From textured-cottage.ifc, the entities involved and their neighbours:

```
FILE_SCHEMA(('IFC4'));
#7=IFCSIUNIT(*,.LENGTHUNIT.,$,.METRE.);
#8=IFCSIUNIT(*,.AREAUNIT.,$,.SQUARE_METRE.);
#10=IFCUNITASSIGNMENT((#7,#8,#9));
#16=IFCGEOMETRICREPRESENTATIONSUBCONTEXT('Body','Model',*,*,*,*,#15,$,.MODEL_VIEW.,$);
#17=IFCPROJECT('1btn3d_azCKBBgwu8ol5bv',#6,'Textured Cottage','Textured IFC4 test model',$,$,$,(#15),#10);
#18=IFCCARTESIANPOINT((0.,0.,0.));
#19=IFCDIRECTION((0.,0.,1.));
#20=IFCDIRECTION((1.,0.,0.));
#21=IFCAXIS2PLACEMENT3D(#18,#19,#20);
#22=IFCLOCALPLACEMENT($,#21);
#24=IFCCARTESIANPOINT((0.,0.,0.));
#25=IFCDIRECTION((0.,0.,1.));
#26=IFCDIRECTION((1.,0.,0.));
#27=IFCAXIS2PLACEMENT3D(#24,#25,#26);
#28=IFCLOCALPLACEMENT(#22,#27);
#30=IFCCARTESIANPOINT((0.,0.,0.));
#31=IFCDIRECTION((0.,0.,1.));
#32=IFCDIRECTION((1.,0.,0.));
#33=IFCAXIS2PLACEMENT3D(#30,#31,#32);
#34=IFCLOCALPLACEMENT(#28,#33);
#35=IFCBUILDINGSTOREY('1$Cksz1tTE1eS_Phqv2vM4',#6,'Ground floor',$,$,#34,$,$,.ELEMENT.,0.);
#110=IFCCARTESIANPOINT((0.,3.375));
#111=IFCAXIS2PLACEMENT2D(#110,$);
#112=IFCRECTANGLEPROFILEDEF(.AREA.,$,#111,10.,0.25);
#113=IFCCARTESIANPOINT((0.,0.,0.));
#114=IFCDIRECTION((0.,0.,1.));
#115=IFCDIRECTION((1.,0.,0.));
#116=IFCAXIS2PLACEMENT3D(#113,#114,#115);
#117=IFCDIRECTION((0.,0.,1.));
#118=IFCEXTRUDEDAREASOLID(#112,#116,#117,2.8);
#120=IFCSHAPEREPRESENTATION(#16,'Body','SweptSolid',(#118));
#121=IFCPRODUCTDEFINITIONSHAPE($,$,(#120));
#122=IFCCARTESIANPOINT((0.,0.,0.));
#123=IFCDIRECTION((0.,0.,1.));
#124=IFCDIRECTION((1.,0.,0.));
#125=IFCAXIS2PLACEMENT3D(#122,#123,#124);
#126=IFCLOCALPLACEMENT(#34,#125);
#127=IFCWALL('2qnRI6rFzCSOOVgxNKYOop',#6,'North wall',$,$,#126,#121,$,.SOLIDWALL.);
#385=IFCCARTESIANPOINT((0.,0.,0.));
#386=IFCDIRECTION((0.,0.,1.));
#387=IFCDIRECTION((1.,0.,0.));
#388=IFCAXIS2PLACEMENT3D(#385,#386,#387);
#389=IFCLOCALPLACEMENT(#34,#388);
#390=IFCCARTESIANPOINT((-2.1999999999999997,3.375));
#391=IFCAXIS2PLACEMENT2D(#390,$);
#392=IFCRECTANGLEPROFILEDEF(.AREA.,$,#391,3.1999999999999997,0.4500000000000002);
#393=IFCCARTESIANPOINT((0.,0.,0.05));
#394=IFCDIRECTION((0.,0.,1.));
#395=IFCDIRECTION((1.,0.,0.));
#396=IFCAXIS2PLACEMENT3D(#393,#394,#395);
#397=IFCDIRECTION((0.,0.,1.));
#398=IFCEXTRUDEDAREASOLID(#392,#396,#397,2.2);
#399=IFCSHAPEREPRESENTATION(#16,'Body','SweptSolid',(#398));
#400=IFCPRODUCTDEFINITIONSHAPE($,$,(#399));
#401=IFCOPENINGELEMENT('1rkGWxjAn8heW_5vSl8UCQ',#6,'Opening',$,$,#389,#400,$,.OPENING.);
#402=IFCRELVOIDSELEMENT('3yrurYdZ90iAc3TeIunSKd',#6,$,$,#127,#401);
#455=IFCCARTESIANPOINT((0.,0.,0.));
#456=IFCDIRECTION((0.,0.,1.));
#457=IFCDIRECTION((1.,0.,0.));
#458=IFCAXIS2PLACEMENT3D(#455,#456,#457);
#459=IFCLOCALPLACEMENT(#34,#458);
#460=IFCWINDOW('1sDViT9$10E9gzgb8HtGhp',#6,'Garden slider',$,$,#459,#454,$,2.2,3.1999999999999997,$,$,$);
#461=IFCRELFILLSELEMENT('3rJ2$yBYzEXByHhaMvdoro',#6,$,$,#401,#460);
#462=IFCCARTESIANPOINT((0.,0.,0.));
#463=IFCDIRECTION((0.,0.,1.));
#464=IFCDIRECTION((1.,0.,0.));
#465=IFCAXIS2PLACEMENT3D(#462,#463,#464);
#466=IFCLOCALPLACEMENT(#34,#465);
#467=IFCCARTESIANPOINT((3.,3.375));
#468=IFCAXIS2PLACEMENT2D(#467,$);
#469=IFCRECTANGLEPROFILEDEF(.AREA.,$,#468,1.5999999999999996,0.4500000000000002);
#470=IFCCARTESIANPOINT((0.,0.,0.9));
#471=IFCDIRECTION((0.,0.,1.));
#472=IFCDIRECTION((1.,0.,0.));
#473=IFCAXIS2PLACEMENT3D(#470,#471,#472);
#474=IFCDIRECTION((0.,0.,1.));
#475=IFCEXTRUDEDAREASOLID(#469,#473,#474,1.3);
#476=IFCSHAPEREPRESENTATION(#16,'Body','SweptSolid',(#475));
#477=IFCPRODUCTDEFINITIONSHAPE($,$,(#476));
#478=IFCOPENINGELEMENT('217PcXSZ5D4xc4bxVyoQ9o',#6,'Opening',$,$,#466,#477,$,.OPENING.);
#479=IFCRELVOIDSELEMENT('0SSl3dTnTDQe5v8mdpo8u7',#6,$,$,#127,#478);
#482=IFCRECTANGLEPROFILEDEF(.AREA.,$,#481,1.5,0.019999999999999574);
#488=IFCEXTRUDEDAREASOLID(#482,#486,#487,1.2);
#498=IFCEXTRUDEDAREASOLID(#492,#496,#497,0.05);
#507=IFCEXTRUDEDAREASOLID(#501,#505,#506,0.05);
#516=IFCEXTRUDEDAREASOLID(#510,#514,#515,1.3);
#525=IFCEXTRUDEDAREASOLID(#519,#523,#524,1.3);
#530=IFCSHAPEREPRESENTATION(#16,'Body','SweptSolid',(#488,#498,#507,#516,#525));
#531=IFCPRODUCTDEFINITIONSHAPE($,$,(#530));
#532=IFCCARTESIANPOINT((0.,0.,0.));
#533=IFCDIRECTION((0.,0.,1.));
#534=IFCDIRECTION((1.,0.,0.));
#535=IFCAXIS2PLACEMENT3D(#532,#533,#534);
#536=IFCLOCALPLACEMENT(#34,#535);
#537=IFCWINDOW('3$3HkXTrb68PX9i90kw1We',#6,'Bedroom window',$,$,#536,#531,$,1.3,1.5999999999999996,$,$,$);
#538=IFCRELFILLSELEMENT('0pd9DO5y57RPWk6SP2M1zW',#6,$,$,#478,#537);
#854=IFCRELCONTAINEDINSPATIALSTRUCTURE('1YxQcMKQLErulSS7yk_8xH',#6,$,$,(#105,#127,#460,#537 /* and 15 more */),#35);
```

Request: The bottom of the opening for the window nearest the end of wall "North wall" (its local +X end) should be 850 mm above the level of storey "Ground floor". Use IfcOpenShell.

```python
import numpy as np
import ifcopenshell
import ifcopenshell.api.geometry
import ifcopenshell.geom
import ifcopenshell.util.element
import ifcopenshell.util.placement
import ifcopenshell.util.shape
import ifcopenshell.util.unit

model = ifcopenshell.open("textured-cottage.ifc")
unit_scale = ifcopenshell.util.unit.calculate_unit_scale(model)

window = model.by_guid("3$3HkXTrb68PX9i90kw1We")
opening = window.FillsVoids[0].RelatingOpeningElement
storey = ifcopenshell.util.element.get_container(window, ifc_class="IfcBuildingStorey")
level = ifcopenshell.util.placement.get_local_placement(storey.ObjectPlacement)[2, 3]

# The opening's origin need not be at the sill, so measure its lowest point.
shape = ifcopenshell.geom.create_shape(ifcopenshell.geom.settings(), opening)
bottom = ifcopenshell.util.shape.get_shape_bottom_elevation(shape, shape.geometry) / unit_scale
dz = level + 0.85 - bottom

shift = np.array([0.0, 0.0, dz])
# The window is not placed relative to its opening, so move both.
for product in (opening, window):
    matrix = ifcopenshell.util.placement.get_local_placement(product.ObjectPlacement)
    matrix[:3, 3] += shift
    ifcopenshell.api.geometry.edit_object_placement(model, product=product, matrix=matrix, is_si=False)

print(f"moved by {dz * unit_scale:+.3f} m")

model.write("textured-cottage_edited.ifc")
```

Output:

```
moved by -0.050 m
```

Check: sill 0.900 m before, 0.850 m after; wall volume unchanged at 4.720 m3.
